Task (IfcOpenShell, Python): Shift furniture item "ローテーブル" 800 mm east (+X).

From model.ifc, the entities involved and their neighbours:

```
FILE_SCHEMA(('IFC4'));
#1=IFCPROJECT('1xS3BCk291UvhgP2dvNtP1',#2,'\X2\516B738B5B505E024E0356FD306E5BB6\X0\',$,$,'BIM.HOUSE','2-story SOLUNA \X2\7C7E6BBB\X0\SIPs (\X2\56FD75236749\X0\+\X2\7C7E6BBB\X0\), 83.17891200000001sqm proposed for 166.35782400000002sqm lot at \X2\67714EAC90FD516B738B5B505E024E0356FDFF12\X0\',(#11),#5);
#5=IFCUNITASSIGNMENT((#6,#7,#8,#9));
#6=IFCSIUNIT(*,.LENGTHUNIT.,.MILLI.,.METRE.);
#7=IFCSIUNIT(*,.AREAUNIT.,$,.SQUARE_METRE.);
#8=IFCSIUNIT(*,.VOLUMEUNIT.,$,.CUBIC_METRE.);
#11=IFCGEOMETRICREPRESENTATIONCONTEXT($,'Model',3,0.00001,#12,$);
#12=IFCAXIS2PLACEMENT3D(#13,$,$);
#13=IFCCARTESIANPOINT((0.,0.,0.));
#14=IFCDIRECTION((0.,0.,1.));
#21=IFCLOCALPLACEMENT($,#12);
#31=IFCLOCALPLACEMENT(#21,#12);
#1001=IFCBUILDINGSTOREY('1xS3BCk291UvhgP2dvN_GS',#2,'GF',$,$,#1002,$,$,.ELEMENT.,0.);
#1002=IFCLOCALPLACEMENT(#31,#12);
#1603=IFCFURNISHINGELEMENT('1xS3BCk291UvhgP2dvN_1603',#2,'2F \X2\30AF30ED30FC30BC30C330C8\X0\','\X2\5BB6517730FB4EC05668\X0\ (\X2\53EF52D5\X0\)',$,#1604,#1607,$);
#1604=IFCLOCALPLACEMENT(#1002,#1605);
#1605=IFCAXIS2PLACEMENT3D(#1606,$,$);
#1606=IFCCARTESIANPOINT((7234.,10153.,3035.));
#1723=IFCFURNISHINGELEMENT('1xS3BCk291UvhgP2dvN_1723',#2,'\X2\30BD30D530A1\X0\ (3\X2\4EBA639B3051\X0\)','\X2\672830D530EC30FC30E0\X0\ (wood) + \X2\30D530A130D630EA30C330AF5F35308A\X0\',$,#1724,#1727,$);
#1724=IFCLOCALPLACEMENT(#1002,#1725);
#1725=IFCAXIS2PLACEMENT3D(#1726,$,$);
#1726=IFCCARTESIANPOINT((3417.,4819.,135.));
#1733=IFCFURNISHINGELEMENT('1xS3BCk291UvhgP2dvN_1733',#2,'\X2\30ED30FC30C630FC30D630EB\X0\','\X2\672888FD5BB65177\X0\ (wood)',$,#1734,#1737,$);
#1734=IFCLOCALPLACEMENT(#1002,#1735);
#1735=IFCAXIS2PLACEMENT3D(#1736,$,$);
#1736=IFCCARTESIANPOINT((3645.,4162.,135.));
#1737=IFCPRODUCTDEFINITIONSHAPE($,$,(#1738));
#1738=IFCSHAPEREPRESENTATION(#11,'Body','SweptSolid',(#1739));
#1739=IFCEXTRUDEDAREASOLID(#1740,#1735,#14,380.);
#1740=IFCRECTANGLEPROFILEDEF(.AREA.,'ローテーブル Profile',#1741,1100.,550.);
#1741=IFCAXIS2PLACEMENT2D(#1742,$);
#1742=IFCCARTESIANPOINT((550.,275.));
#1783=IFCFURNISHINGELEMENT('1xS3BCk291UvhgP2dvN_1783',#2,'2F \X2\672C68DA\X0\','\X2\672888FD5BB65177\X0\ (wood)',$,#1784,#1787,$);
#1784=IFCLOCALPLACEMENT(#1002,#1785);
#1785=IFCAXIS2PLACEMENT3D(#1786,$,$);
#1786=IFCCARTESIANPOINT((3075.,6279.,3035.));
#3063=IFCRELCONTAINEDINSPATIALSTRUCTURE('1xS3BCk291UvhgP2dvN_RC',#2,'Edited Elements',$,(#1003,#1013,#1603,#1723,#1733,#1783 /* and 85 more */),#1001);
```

```python
import ifcopenshell
import ifcopenshell.api.geometry
import ifcopenshell.util.placement
import ifcopenshell.util.unit

model = ifcopenshell.open("model.ifc")
unit_scale = ifcopenshell.util.unit.calculate_unit_scale(model)

item = model.by_guid("1xS3BCk291UvhgP2dvN_1733")
matrix = ifcopenshell.util.placement.get_local_placement(item.ObjectPlacement)
matrix[0, 3] += 0.8 / unit_scale
ifcopenshell.api.geometry.edit_object_placement(model, product=item, matrix=matrix, is_si=False)

print(ifcopenshell.util.placement.get_local_placement(item.ObjectPlacement).round(3) + 0.0)

model.write("model_updated.ifc")
```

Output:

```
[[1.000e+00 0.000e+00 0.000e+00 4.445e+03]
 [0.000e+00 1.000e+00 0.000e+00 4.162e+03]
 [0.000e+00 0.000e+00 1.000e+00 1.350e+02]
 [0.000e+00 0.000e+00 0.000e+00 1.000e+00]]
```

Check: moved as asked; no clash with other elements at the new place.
